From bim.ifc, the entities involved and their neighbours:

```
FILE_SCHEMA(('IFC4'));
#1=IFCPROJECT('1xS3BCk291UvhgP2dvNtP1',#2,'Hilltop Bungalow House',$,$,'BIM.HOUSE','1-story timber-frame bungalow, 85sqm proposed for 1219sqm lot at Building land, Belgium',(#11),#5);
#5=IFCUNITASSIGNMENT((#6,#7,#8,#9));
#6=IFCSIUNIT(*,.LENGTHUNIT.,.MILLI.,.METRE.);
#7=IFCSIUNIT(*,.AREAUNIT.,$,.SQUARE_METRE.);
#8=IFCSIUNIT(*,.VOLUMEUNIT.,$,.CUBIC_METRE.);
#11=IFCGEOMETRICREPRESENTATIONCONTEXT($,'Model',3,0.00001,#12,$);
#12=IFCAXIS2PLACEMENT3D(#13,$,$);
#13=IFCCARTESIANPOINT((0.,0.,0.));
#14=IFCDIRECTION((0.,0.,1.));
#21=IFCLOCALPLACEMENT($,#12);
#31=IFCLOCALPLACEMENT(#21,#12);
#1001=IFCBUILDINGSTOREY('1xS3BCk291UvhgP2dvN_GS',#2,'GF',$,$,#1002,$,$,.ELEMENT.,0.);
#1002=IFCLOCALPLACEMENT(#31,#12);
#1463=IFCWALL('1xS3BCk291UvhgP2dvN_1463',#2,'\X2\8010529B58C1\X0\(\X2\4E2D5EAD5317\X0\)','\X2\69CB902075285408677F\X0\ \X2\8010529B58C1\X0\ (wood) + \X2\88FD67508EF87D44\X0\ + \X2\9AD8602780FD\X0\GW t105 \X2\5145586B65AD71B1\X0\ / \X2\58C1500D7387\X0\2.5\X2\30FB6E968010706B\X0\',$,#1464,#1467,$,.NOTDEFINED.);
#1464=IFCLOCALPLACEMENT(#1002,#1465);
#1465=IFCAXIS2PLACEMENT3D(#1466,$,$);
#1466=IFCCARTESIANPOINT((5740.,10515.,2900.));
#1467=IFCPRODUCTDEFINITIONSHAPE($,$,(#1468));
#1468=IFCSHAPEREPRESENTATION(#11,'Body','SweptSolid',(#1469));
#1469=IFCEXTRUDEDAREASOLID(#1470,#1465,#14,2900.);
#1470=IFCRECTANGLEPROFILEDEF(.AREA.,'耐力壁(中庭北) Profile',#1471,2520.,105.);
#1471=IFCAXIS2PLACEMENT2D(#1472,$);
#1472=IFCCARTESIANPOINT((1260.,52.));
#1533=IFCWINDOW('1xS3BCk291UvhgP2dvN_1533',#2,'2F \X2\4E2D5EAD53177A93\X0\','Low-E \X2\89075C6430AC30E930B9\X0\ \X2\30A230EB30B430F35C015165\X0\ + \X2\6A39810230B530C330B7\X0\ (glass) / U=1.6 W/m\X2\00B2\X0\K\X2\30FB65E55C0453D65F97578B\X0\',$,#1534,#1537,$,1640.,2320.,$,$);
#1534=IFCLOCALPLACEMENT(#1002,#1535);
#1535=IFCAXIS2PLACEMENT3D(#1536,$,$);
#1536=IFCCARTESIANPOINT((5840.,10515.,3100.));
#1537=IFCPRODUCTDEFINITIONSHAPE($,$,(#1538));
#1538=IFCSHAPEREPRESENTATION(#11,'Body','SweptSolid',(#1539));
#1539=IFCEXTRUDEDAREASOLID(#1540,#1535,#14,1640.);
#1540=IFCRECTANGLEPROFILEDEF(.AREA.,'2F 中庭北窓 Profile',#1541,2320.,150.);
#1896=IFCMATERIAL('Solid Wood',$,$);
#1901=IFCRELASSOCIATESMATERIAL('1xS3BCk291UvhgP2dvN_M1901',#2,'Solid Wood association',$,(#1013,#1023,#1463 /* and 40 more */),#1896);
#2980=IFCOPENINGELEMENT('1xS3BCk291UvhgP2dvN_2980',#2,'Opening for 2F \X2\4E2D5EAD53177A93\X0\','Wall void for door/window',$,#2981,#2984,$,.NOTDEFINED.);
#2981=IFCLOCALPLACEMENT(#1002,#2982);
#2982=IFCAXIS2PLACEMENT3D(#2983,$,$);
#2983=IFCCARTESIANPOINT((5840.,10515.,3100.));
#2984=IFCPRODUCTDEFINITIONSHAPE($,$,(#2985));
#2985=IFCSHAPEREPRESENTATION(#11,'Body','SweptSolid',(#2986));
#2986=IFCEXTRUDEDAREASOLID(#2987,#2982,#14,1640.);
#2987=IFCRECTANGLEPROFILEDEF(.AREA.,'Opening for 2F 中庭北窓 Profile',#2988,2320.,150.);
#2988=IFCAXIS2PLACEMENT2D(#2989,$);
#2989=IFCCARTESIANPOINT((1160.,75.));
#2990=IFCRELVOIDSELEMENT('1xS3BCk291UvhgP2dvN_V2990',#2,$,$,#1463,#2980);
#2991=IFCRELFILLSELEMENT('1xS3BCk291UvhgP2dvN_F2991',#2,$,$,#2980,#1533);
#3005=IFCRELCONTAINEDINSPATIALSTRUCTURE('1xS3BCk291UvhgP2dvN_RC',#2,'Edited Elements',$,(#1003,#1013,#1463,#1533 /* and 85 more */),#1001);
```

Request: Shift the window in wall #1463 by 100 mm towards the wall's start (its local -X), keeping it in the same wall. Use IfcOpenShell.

```python
import ifcopenshell
import ifcopenshell.api.geometry
import ifcopenshell.util.placement
import ifcopenshell.util.unit

model = ifcopenshell.open("bim.ifc")
unit_scale = ifcopenshell.util.unit.calculate_unit_scale(model)

window = model.by_guid("1xS3BCk291UvhgP2dvN_1533")
opening = window.FillsVoids[0].RelatingOpeningElement
wall = opening.VoidsElements[0].RelatingBuildingElement

wall_matrix = ifcopenshell.util.placement.get_local_placement(wall.ObjectPlacement)
shift = wall_matrix[:3, 0] * -0.1 / unit_scale
before = ifcopenshell.util.placement.get_local_placement(window.ObjectPlacement)[:3, 3].copy()

# The window is not placed relative to its opening, so move both.
for product in (opening, window):
    matrix = ifcopenshell.util.placement.get_local_placement(product.ObjectPlacement)
    matrix[:3, 3] += shift
    ifcopenshell.api.geometry.edit_object_placement(model, product=product, matrix=matrix, is_si=False)

after = ifcopenshell.util.placement.get_local_placement(window.ObjectPlacement)[:3, 3]
print("window moved by", (after - before).round(3) + 0.0)

model.write("bim-out.ifc")
```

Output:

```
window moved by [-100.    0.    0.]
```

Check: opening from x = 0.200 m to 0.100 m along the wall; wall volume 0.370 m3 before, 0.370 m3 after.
